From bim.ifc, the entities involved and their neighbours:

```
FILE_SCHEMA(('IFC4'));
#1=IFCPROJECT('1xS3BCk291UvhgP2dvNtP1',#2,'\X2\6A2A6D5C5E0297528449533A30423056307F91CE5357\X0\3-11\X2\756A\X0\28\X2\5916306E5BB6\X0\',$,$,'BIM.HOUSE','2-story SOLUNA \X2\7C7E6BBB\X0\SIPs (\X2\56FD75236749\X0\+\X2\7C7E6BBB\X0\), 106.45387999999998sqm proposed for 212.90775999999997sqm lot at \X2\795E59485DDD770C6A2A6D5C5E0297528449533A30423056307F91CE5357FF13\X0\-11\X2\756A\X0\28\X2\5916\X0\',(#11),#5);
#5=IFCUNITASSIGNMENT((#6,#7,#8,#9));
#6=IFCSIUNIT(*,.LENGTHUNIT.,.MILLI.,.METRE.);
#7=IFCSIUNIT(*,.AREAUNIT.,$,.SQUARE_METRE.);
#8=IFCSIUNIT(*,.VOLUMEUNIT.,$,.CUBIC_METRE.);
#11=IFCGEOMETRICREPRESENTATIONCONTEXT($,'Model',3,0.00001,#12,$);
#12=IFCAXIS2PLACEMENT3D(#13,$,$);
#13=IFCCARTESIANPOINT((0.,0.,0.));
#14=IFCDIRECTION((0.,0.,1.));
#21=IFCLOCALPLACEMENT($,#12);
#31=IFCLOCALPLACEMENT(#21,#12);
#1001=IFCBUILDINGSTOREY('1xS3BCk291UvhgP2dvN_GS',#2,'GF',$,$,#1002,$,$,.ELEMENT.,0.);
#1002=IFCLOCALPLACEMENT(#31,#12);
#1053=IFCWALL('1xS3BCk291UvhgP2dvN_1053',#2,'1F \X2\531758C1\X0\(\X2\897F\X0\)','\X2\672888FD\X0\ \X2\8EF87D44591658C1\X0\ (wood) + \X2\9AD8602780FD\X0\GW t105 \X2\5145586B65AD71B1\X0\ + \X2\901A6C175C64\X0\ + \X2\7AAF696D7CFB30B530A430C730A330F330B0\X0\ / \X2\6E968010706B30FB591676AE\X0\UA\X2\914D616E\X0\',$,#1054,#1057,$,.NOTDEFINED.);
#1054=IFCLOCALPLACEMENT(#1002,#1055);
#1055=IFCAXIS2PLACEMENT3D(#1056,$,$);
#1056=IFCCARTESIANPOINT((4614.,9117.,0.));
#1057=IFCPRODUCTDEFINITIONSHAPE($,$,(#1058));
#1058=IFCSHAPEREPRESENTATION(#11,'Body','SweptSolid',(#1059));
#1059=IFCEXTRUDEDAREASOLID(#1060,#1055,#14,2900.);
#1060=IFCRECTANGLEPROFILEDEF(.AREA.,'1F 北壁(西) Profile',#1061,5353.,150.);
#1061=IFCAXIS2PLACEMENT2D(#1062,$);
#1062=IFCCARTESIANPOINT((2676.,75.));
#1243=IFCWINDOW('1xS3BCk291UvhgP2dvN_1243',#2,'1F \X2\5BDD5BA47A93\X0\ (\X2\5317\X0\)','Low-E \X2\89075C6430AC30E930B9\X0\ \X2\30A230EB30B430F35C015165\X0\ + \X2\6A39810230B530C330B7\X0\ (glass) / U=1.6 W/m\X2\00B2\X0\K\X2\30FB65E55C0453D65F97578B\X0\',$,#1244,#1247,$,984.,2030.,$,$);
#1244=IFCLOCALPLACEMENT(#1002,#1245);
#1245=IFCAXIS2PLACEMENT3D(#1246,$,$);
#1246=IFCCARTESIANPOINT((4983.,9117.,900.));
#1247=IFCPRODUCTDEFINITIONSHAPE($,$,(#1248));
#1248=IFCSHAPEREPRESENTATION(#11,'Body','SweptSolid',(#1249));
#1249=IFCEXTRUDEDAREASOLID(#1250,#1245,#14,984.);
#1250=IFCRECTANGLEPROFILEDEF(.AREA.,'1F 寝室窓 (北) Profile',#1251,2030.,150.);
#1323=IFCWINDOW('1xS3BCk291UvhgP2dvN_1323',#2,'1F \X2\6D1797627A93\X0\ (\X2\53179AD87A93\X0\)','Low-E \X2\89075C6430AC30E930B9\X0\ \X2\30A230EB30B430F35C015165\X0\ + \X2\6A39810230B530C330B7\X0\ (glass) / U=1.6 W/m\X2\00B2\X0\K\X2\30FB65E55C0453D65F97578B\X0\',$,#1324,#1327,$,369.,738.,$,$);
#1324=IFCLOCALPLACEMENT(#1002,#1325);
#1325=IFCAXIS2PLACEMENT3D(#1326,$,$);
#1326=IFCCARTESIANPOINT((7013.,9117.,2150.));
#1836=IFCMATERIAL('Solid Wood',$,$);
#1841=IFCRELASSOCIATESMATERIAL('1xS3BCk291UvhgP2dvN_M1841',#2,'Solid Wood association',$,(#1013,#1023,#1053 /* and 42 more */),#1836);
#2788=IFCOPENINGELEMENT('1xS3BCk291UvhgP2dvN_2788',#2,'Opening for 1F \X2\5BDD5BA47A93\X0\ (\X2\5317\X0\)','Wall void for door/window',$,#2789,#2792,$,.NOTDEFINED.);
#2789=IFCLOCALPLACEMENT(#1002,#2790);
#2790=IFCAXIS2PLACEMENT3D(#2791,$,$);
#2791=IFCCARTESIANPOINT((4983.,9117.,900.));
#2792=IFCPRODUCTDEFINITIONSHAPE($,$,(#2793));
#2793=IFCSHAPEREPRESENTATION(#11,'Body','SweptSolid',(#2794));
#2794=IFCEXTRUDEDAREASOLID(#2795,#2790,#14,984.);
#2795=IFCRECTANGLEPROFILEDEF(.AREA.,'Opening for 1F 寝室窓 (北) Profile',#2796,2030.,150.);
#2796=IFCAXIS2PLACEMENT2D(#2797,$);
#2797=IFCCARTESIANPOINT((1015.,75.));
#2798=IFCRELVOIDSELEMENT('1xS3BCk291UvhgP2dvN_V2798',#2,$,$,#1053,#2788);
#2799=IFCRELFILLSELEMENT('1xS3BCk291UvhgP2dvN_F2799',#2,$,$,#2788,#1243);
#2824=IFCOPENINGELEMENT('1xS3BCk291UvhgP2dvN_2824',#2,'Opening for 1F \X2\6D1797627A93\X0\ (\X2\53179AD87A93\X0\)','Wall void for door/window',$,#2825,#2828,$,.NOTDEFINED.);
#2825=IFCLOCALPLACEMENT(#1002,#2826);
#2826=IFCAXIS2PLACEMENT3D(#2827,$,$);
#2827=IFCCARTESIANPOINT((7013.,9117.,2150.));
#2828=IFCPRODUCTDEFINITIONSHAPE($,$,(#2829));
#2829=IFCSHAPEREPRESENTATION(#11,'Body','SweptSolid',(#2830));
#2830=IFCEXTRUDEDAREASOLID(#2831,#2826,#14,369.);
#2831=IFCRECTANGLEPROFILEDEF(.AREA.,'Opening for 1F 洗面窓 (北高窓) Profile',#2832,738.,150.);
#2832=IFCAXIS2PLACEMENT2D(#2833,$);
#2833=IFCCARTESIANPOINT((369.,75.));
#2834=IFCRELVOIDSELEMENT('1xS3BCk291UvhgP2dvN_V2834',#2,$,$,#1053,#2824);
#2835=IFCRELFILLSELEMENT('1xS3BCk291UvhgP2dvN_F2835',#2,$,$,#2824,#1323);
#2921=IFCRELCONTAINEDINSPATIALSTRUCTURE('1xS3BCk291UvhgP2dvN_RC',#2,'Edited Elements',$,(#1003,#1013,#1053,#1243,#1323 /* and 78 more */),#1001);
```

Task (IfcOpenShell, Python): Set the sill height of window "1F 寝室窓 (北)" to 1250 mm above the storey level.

```python
import numpy as np
import ifcopenshell
import ifcopenshell.api.geometry
import ifcopenshell.geom
import ifcopenshell.util.element
import ifcopenshell.util.placement
import ifcopenshell.util.shape
import ifcopenshell.util.unit

model = ifcopenshell.open("bim.ifc")
unit_scale = ifcopenshell.util.unit.calculate_unit_scale(model)

window = model.by_guid("1xS3BCk291UvhgP2dvN_1243")
opening = window.FillsVoids[0].RelatingOpeningElement
storey = ifcopenshell.util.element.get_container(window, ifc_class="IfcBuildingStorey")
level = ifcopenshell.util.placement.get_local_placement(storey.ObjectPlacement)[2, 3]

# The opening's origin need not be at the sill, so measure its lowest point.
shape = ifcopenshell.geom.create_shape(ifcopenshell.geom.settings(), opening)
bottom = ifcopenshell.util.shape.get_shape_bottom_elevation(shape, shape.geometry) / unit_scale
dz = level + 1250.0 - bottom

shift = np.array([0.0, 0.0, dz])
# The window is not placed relative to its opening, so move both.
for product in (opening, window):
    matrix = ifcopenshell.util.placement.get_local_placement(product.ObjectPlacement)
    matrix[:3, 3] += shift
    ifcopenshell.api.geometry.edit_object_placement(model, product=product, matrix=matrix, is_si=False)

print(f"moved by {dz * unit_scale:+.3f} m")

model.write("bim_v2.ifc")
```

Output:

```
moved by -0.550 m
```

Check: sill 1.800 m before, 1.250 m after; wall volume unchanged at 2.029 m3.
